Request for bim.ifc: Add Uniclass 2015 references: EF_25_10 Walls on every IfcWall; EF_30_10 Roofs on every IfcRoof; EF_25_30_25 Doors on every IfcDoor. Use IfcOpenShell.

First a look at what the model holds.

```python
import ifcopenshell

model = ifcopenshell.open("bim.ifc")
print(model.schema)
print("classifications:", [c.Name for c in model.by_type("IfcClassification")])
for ifc_class in ("IfcDoor", "IfcRoof", "IfcStair", "IfcWall", "IfcWindow"):
    print(ifc_class, len(model.by_type(ifc_class)))
```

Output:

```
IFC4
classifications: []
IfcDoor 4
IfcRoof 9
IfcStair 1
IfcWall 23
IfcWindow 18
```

```python
import ifcopenshell
import ifcopenshell.api.classification

model = ifcopenshell.open("bim.ifc")

system = ifcopenshell.api.classification.add_classification(model, classification="Uniclass 2015")

codes = {
    "IfcWall": ("EF_25_10", "Walls"),
    "IfcRoof": ("EF_30_10", "Roofs"),
    "IfcDoor": ("EF_25_30_25", "Doors"),
}
for ifc_class, (code, name) in codes.items():
    products = model.by_type(ifc_class)
    ifcopenshell.api.classification.add_reference(
        model, products=products, classification=system, identification=code, name=name
    )
    print(code, len(products))

model.write("bim-out.ifc")
```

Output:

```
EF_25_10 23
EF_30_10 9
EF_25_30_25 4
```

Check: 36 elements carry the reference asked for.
